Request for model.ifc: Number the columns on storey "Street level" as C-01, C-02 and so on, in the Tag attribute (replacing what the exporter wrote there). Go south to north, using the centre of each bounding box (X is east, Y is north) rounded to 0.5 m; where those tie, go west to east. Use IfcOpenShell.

First a look at what the model holds.

```python
import ifcopenshell
import ifcopenshell.util.element
import ifcopenshell.util.placement

model = ifcopenshell.open("model.ifc")
print(model.schema)
storey = next(s for s in model.by_type("IfcBuildingStorey") if s.Name == "Street level")
columns = [e for e in ifcopenshell.util.element.get_decomposition(storey) if e.is_a("IfcColumn")]
for e in sorted(columns, key=lambda e: e.id()):
    origin = ifcopenshell.util.placement.get_local_placement(e.ObjectPlacement)[:3, 3]
    print(e.id(), e.Tag, e.Name, origin.round(2) + 0.0, sep=" | ")
```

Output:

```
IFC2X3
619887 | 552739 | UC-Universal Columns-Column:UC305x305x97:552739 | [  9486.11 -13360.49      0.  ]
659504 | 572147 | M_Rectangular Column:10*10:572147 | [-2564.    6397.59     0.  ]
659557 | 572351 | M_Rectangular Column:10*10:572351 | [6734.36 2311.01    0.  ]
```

```python
import ifcopenshell
import ifcopenshell.geom
import ifcopenshell.util.element
import ifcopenshell.util.shape

model = ifcopenshell.open("model.ifc")
settings = ifcopenshell.geom.settings()
settings.set("use-world-coords", True)


def centre(element):
    shape = ifcopenshell.geom.create_shape(settings, element)
    return ifcopenshell.util.shape.get_bbox_centroid(shape.geometry)


storey = next(s for s in model.by_type("IfcBuildingStorey") if s.Name == "Street level")
columns = [e for e in ifcopenshell.util.element.get_decomposition(storey) if e.is_a("IfcColumn")]

# Insertion points can sit at a corner or the storey origin, so sort by the geometry (in metres).
centres = {e: centre(e) for e in columns}
columns.sort(key=lambda e: (round(centres[e][1] / 0.5), centres[e][0]))

for i, e in enumerate(columns, start=1):
    number = f"C-{i:02d}"
    e.Tag = number
    print(e.id(), number)

model.write("model_v2.ifc")
```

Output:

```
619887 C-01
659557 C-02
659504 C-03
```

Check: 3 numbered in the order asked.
